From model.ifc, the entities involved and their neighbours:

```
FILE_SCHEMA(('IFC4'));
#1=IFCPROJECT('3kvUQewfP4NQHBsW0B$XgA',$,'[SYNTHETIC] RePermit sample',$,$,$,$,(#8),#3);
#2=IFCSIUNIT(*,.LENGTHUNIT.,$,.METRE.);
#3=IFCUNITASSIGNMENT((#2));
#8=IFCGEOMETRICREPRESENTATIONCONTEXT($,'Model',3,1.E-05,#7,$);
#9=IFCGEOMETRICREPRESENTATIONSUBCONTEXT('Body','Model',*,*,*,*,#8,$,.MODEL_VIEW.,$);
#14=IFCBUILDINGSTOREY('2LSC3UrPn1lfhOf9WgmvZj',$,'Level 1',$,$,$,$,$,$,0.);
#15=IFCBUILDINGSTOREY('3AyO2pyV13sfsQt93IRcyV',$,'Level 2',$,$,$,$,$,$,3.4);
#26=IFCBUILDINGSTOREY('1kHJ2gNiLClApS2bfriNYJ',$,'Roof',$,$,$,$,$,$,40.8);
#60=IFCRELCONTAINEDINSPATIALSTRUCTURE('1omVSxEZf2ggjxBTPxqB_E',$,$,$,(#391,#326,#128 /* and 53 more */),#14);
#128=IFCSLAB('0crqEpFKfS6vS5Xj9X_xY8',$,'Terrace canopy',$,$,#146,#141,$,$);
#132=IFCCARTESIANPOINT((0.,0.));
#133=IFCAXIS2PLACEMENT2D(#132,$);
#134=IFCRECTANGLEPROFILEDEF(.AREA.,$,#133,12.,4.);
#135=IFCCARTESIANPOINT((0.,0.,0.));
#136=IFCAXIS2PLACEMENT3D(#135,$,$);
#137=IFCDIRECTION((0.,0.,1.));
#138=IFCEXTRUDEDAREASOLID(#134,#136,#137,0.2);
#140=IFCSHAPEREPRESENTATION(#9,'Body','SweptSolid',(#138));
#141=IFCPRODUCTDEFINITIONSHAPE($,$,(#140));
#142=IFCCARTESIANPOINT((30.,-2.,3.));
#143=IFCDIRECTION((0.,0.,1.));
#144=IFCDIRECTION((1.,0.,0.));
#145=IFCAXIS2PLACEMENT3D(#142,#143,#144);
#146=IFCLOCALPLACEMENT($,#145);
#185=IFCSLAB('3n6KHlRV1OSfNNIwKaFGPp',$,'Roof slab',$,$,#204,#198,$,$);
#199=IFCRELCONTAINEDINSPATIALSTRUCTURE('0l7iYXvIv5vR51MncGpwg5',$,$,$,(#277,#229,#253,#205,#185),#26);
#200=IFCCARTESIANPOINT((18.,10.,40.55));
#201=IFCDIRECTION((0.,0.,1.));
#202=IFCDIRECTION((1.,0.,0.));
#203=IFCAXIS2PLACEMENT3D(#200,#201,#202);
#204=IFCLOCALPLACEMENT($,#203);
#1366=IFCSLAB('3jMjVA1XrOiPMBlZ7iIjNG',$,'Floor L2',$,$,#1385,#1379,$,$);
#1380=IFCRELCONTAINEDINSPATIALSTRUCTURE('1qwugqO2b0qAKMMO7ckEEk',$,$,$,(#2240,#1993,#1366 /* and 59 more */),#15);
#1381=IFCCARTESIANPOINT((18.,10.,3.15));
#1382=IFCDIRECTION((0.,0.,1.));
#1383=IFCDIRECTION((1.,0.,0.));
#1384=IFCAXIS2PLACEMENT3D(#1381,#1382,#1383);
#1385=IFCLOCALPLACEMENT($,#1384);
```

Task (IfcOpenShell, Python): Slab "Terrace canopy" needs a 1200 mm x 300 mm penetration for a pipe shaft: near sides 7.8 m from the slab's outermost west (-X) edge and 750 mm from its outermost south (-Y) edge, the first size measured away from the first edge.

```python
import numpy as np
import ifcopenshell
import ifcopenshell.api.feature
import ifcopenshell.api.geometry
import ifcopenshell.api.root
import ifcopenshell.geom
import ifcopenshell.util.placement
import ifcopenshell.util.representation
import ifcopenshell.util.shape
import ifcopenshell.util.unit

model = ifcopenshell.open("model.ifc")
unit_scale = ifcopenshell.util.unit.calculate_unit_scale(model)
settings = ifcopenshell.geom.settings()


def volume(element):
    """Net volume in cubic metres, openings subtracted."""
    shape = ifcopenshell.geom.create_shape(settings, element)
    return ifcopenshell.util.shape.get_volume(shape.geometry)


slab = model.by_id(128)
before = volume(slab)

# Extent in the slab's own axes, in metres. The edges named are its -X and -Y sides.
slab_shape = ifcopenshell.geom.create_shape(settings, slab)
vertices = ifcopenshell.util.shape.get_vertices(slab_shape.geometry)
x_min, y_min, bottom = vertices.min(axis=0)
top = vertices[:, 2].max()

opening = ifcopenshell.api.root.create_entity(model, ifc_class="IfcOpeningElement", name="Pipe shaft opening", predefined_type="OPENING")
context = ifcopenshell.util.representation.get_context(model, "Model", "Body", "MODEL_VIEW")
width, depth = 1.2, 0.3
outline = [(0.0, 0.0), (width, 0.0), (width, depth), (0.0, depth), (0.0, 0.0)]
# Overshoot both faces by 50 mm so the cut is clean.
shape = ifcopenshell.api.geometry.add_slab_representation(
    model, context=context, depth=top - bottom + 0.1, polyline=outline
)
ifcopenshell.api.geometry.assign_representation(model, product=opening, representation=shape)

matrix = ifcopenshell.util.placement.get_local_placement(slab.ObjectPlacement)
matrix[:, 3] = matrix @ np.append(np.array([x_min + 7.8, y_min + 0.75, bottom - 0.05]) / unit_scale, 1.0)
ifcopenshell.api.geometry.edit_object_placement(model, product=opening, matrix=matrix, is_si=False)
ifcopenshell.api.feature.add_feature(model, feature=opening, element=slab)

after = volume(slab)

print(f"slab volume {before:.3f} -> {after:.3f} m3")

model.write("model_edited.ifc")
```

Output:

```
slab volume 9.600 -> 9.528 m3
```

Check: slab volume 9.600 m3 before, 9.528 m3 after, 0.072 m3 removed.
